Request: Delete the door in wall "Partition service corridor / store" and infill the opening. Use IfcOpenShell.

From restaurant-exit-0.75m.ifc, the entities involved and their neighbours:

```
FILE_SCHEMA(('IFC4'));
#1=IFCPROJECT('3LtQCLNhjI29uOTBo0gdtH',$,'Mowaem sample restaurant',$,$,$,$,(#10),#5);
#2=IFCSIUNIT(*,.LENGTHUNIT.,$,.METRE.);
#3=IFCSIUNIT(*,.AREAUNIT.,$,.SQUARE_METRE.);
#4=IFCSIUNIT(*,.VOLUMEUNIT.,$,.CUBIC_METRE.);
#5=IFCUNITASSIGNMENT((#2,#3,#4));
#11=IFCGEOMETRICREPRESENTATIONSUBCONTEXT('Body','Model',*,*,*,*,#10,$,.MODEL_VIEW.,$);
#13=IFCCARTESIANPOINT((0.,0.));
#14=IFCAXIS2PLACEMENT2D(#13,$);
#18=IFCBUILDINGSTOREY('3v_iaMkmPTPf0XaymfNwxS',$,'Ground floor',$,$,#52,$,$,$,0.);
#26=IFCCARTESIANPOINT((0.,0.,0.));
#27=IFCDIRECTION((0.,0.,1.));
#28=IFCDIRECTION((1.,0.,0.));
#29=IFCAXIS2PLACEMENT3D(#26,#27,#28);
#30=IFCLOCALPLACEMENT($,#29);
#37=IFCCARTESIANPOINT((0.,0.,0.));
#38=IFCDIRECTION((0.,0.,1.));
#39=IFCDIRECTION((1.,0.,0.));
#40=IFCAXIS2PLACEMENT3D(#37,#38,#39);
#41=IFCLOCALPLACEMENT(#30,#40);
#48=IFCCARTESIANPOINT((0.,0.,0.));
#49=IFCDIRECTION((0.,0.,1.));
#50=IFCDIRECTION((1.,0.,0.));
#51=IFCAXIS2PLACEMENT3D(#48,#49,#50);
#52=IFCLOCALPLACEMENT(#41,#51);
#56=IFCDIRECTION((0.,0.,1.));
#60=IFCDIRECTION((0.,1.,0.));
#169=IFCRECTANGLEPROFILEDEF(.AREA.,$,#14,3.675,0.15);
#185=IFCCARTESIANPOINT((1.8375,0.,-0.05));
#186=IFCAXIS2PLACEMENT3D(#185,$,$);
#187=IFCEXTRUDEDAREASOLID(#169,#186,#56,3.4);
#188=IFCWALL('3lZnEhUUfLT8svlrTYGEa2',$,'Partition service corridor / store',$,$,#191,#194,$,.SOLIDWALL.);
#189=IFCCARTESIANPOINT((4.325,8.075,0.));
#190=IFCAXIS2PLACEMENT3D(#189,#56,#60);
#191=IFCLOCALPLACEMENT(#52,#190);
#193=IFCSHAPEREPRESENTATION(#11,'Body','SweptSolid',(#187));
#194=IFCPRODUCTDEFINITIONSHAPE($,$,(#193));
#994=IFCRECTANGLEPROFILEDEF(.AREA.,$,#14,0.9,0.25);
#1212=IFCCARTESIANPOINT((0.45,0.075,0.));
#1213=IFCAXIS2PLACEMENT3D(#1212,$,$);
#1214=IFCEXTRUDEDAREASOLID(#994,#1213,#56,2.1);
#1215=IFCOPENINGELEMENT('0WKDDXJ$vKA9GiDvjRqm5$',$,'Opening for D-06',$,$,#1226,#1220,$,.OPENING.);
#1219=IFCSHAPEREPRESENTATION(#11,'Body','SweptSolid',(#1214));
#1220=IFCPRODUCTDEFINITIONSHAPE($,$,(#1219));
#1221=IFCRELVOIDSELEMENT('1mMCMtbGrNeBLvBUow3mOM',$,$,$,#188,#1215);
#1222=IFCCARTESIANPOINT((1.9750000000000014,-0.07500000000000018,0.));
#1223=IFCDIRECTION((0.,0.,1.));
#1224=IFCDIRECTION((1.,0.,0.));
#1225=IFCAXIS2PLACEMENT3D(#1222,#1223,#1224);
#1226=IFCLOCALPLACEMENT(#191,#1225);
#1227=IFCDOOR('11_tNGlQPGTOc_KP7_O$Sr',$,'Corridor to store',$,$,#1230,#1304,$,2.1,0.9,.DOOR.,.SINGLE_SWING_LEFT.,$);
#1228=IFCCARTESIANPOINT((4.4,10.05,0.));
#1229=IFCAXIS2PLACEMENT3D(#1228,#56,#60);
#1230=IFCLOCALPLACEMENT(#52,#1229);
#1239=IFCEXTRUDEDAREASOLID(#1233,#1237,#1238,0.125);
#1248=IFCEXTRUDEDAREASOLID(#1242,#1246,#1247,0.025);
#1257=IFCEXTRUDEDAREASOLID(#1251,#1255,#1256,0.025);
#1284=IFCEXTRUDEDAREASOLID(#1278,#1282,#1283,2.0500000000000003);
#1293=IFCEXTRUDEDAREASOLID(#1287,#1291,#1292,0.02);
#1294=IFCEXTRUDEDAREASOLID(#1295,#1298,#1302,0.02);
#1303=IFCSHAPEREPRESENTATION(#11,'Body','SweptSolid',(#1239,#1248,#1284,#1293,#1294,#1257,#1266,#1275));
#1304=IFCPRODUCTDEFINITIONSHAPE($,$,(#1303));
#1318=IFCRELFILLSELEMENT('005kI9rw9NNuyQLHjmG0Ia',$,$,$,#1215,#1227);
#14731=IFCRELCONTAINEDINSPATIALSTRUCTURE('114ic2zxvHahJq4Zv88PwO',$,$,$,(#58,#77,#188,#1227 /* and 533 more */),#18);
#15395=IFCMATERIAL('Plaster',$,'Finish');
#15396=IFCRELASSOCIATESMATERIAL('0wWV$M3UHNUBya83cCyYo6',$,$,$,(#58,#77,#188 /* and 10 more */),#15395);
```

```python
import ifcopenshell
import ifcopenshell.api.feature
import ifcopenshell.api.root
import ifcopenshell.geom
import ifcopenshell.util.shape

model = ifcopenshell.open("restaurant-exit-0.75m.ifc")
settings = ifcopenshell.geom.settings()


def volume(element):
    """Net volume in cubic metres, openings subtracted."""
    shape = ifcopenshell.geom.create_shape(settings, element)
    return ifcopenshell.util.shape.get_volume(shape.geometry)


door = model.by_guid("11_tNGlQPGTOc_KP7_O$Sr")
opening = door.FillsVoids[0].RelatingOpeningElement
wall = opening.VoidsElements[0].RelatingBuildingElement
before = volume(wall)

ifcopenshell.api.root.remove_product(model, product=door)
ifcopenshell.api.feature.remove_feature(model, feature=opening)

after = volume(wall)

print(f"wall volume {before:.3f} -> {after:.3f} m3")

model.write("restaurant-exit-0.75m_edited.ifc")
```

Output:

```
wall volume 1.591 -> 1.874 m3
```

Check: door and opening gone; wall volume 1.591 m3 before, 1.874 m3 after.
